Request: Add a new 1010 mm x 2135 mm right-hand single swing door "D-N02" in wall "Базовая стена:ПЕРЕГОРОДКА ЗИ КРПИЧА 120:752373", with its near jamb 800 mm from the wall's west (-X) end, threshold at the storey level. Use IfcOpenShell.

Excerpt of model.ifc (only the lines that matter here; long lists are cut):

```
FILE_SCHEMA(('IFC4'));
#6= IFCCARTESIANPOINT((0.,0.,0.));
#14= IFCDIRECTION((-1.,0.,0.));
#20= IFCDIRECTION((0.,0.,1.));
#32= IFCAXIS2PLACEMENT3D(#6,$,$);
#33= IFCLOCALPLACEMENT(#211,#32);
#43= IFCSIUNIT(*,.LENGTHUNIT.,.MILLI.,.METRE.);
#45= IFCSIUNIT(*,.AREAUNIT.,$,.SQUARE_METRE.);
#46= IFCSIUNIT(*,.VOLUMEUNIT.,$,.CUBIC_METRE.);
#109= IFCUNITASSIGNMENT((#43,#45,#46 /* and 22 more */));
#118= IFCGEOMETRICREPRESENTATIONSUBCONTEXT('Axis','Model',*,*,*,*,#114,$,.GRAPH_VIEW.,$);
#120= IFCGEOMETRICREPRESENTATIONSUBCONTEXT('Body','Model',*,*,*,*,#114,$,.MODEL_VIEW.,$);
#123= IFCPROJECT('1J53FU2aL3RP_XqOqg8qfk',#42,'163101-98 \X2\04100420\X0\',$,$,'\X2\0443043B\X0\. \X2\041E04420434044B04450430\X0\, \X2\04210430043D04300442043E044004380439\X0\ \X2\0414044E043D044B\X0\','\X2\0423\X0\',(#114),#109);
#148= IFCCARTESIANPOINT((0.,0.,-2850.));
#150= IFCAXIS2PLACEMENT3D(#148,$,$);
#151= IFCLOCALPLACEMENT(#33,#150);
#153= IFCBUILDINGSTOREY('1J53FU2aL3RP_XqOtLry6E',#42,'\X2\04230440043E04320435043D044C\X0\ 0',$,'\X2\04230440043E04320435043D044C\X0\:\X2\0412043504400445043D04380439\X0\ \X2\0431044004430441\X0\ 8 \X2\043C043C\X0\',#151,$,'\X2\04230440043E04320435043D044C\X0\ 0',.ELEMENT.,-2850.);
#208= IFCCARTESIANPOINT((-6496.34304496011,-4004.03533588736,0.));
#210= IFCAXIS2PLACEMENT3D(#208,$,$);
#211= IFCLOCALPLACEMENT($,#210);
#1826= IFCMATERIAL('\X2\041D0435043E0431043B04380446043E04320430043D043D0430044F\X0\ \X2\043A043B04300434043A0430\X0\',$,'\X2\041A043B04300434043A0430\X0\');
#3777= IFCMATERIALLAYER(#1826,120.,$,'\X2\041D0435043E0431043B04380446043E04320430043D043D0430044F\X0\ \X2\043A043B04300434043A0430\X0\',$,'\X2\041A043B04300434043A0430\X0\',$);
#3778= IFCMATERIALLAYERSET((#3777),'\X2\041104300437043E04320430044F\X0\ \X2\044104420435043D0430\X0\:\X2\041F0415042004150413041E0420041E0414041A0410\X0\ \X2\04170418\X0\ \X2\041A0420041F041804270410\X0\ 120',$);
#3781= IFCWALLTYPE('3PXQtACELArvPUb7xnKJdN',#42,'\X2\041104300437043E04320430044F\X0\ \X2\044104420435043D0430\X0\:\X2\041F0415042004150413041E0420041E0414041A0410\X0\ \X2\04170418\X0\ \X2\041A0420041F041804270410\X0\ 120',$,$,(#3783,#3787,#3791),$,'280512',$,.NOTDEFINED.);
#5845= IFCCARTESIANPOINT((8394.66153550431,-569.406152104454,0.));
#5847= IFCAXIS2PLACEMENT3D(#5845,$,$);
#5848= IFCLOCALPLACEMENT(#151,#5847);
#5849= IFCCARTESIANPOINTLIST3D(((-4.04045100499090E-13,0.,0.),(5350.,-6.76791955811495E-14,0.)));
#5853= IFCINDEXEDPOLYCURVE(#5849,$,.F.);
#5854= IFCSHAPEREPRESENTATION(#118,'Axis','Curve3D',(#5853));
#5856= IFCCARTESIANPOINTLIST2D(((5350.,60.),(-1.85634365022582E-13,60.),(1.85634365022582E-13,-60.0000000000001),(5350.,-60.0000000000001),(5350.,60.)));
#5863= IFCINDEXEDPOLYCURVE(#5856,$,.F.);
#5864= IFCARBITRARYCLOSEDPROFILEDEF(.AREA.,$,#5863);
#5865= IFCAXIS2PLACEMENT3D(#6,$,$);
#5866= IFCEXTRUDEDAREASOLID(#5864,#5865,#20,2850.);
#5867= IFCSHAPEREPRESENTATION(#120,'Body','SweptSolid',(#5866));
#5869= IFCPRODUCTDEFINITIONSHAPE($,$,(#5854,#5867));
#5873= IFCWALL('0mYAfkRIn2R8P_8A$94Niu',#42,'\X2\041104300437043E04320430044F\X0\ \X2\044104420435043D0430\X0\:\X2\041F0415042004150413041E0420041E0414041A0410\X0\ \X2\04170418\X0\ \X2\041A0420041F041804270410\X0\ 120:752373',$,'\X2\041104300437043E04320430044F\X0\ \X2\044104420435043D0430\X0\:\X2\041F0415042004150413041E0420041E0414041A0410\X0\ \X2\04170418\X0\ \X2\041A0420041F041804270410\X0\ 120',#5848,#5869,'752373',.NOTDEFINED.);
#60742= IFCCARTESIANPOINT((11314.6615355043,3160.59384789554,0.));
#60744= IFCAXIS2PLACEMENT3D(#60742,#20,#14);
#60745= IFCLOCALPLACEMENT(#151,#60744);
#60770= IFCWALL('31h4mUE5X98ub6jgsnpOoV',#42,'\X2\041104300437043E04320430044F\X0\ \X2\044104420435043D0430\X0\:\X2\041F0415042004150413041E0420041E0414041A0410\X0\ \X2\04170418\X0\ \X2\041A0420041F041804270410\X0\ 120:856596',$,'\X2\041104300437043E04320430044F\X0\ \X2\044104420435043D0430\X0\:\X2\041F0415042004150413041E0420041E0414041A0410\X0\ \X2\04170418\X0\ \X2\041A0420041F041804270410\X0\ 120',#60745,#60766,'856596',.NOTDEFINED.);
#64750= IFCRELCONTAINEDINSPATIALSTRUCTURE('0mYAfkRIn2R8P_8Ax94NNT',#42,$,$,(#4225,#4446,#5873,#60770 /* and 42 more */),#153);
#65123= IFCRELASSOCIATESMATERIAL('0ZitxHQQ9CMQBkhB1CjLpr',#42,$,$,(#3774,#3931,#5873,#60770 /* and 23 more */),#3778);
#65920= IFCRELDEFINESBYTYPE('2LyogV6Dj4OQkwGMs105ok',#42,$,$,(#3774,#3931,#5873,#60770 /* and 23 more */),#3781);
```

```python
import numpy as np
import ifcopenshell
import ifcopenshell.api.feature
import ifcopenshell.api.geometry
import ifcopenshell.api.root
import ifcopenshell.api.spatial
import ifcopenshell.geom
import ifcopenshell.util.element
import ifcopenshell.util.placement
import ifcopenshell.util.representation
import ifcopenshell.util.shape
import ifcopenshell.util.unit

model = ifcopenshell.open("model.ifc")
unit_scale = ifcopenshell.util.unit.calculate_unit_scale(model)
settings = ifcopenshell.geom.settings()


def volume(element):
    """Net volume in cubic metres, openings subtracted."""
    shape = ifcopenshell.geom.create_shape(settings, element)
    return ifcopenshell.util.shape.get_volume(shape.geometry)


wall = model.by_id(5873)
storey = ifcopenshell.util.element.get_container(wall, ifc_class="IfcBuildingStorey")
context = ifcopenshell.util.representation.get_context(model, "Model", "Body", "MODEL_VIEW")
before = volume(wall)

width, height, from_end, sill = 1.01, 2.135, 0.8, 0.0  # metres

# The wall runs along its own X axis, and the end named is its -X end.
wall_shape = ifcopenshell.geom.create_shape(settings, wall)
x, y, z = ifcopenshell.util.shape.get_vertices(wall_shape.geometry).T
start = x.min() + from_end
face, thickness = float(y.min()), float(y.max() - y.min())
wall_matrix = ifcopenshell.util.placement.get_local_placement(wall.ObjectPlacement)
level = ifcopenshell.util.placement.get_local_placement(storey.ObjectPlacement)[2, 3]


def in_wall(x, y):
    """Placement at x, y metres in the wall's axes, at sill height."""
    matrix = wall_matrix.copy()
    matrix[:, 3] = wall_matrix @ np.array([x / unit_scale, y / unit_scale, 0.0, 1.0])
    matrix[2, 3] = level + sill / unit_scale
    return matrix


# Opening: a box that overshoots both wall faces by 50 mm.
opening = ifcopenshell.api.root.create_entity(model, ifc_class="IfcOpeningElement", predefined_type="OPENING")
box = ifcopenshell.api.geometry.add_wall_representation(
    model, context=context, length=width, height=height, thickness=thickness + 0.1
)
ifcopenshell.api.geometry.assign_representation(model, product=opening, representation=box)
ifcopenshell.api.geometry.edit_object_placement(model, product=opening, matrix=in_wall(start, face - 0.05), is_si=False)
ifcopenshell.api.feature.add_feature(model, feature=opening, element=wall)

door = ifcopenshell.api.root.create_entity(model, ifc_class="IfcDoor", name="D-N02", predefined_type="DOOR")
door.OverallWidth, door.OverallHeight = width / unit_scale, height / unit_scale
door.OperationType = "SINGLE_SWING_RIGHT"
body = ifcopenshell.api.geometry.add_door_representation(
    model,
    context=context,
    overall_width=door.OverallWidth,
    overall_height=door.OverallHeight,
    operation_type="SINGLE_SWING_RIGHT",
    lining_properties={"LiningDepth": thickness / unit_scale, "ThresholdDepth": thickness / unit_scale},
)
ifcopenshell.api.geometry.assign_representation(model, product=door, representation=body)
ifcopenshell.api.spatial.assign_container(model, products=[door], relating_structure=storey)
ifcopenshell.api.feature.add_filling(model, opening=opening, element=door)

# The lining spans the wall, so the door starts at the wall face.
ifcopenshell.api.geometry.edit_object_placement(model, product=door, matrix=in_wall(start, face), is_si=False)

after = volume(wall)

print(f"wall volume {before:.3f} -> {after:.3f} m3")

model.write("model-out.ifc")
```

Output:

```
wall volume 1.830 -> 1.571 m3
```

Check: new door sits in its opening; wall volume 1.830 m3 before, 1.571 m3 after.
